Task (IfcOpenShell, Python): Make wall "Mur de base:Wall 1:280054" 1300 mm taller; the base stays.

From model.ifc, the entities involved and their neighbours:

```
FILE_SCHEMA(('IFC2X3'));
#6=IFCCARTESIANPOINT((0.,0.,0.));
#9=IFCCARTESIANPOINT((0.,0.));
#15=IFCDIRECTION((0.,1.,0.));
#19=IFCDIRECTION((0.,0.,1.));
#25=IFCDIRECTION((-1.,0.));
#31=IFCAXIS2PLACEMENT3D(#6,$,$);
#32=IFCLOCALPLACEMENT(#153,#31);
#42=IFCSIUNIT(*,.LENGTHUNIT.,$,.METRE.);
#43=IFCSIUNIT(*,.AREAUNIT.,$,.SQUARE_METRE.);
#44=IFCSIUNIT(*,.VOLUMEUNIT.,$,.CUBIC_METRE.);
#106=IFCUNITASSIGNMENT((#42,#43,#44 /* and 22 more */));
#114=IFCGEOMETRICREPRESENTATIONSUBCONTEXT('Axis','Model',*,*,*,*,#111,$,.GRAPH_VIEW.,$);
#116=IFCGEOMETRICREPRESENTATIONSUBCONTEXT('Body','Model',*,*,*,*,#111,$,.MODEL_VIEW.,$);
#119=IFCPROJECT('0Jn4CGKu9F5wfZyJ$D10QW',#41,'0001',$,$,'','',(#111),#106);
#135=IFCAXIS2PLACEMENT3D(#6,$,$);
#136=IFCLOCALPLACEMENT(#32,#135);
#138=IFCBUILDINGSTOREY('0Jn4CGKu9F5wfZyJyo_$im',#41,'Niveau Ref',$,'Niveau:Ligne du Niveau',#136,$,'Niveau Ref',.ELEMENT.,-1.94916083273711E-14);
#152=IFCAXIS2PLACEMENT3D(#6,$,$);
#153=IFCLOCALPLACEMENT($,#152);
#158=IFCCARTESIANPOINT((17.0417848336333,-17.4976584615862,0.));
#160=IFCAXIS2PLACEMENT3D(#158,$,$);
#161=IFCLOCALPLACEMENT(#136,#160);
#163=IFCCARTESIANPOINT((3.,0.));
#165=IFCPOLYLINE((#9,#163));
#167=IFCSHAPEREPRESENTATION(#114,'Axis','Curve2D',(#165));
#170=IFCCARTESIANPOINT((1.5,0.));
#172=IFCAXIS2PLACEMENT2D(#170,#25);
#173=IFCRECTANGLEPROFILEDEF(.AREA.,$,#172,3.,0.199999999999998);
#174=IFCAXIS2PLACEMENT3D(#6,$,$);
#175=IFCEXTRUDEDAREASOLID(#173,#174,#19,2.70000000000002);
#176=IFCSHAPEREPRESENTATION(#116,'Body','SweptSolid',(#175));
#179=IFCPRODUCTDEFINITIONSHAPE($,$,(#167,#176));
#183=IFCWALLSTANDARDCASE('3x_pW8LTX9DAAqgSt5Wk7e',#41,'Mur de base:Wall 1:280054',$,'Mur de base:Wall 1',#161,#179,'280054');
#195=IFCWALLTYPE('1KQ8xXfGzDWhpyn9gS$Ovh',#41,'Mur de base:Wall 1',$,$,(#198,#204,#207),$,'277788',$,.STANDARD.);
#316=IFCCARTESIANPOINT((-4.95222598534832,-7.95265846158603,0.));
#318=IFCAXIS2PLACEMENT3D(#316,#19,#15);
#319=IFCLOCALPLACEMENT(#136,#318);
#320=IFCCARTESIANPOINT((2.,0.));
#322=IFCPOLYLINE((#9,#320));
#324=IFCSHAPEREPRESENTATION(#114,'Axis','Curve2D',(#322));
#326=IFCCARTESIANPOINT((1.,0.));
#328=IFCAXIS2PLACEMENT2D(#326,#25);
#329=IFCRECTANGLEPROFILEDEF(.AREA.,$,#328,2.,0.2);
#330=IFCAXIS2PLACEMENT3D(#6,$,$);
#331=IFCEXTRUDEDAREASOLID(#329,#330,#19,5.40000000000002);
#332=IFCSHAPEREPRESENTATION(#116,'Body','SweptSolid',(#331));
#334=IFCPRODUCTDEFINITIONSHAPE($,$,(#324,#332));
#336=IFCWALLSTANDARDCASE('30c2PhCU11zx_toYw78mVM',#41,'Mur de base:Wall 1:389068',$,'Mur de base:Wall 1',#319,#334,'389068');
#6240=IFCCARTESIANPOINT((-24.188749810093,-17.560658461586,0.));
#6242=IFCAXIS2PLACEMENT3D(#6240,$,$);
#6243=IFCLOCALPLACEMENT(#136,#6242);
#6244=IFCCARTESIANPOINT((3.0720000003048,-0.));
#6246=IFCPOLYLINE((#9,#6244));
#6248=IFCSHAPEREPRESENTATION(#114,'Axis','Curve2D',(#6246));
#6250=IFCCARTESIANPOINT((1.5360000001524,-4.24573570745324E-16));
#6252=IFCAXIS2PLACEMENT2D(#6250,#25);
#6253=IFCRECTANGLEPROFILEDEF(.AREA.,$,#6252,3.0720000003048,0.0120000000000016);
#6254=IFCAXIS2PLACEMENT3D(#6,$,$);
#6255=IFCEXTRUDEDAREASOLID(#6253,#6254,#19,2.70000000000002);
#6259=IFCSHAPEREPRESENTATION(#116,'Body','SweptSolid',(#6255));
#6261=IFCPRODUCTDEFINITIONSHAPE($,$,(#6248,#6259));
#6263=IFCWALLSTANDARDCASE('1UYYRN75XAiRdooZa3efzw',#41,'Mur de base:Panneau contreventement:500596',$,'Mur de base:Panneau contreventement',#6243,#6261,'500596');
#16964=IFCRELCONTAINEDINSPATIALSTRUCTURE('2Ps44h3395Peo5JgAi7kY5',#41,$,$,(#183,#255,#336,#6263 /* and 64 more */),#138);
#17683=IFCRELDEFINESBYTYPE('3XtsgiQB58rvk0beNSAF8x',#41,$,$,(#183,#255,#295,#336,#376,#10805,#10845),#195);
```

```python
import ifcopenshell
import ifcopenshell.geom
import ifcopenshell.util.representation
import ifcopenshell.util.shape

model = ifcopenshell.open("model.ifc")
settings = ifcopenshell.geom.settings()


def volume(element):
    """Net volume in cubic metres, openings subtracted."""
    shape = ifcopenshell.geom.create_shape(settings, element)
    return ifcopenshell.util.shape.get_volume(shape.geometry)


wall = model.by_id(183)
before = volume(wall)

body = ifcopenshell.util.representation.get_representation(wall, "Model", "Body")
solid = body.Items[0]
old_height = solid.Depth
solid.Depth += 1.3
after = volume(wall)

print(f"height {old_height:g} -> {solid.Depth:g}, volume {before:.3f} -> {after:.3f} m3")

model.write("model_rev.ifc")
```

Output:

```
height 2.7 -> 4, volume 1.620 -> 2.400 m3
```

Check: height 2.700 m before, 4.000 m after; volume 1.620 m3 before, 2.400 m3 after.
